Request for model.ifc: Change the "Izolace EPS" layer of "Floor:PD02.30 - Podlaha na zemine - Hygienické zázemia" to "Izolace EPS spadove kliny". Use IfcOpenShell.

First a look at what the model holds.

```python
import ifcopenshell
import ifcopenshell.util.element

model = ifcopenshell.open("model.ifc")
print(model.schema)
for layer_set in model.by_type("IfcMaterialLayerSet"):
    if layer_set.LayerSetName == "Floor:PD02.30 - Podlaha na zemine - Hygienické zázemia":
        for layer in layer_set.MaterialLayers:
            print(layer.id(), layer.Material and layer.Material.Name, layer.LayerThickness, sep=" | ")
        print(len(ifcopenshell.util.element.get_elements_by_material(model, layer_set)), "elements and types use it")
print(sorted(m.Name for m in model.by_type("IfcMaterial") if m.Name)[:60])
```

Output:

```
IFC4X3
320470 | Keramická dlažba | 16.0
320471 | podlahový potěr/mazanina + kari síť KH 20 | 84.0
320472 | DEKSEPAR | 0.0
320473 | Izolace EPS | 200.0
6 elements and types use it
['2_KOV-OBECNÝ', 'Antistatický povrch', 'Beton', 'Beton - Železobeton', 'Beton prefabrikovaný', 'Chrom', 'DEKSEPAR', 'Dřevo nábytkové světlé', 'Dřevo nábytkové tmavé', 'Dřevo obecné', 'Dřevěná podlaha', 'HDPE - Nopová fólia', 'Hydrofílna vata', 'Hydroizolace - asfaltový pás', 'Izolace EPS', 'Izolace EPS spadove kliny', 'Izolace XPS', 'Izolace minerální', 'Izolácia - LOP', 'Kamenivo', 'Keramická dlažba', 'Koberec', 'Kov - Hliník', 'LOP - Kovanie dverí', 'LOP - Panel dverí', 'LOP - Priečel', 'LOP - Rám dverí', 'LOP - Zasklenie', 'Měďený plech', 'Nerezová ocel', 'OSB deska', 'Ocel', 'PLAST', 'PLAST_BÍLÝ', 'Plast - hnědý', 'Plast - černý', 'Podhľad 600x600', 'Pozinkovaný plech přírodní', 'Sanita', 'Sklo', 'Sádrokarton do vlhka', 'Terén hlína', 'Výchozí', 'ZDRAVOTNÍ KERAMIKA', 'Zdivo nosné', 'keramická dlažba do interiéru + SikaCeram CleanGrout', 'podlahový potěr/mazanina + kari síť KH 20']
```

```python
import ifcopenshell
import ifcopenshell.api.material

model = ifcopenshell.open("model.ifc")

layer_set = next(s for s in model.by_type("IfcMaterialLayerSet") if s.LayerSetName == "Floor:PD02.30 - Podlaha na zemine - Hygienické zázemia")
layer = next(l for l in layer_set.MaterialLayers if l.Material and l.Material.Name == "Izolace EPS")
material = next(m for m in model.by_type("IfcMaterial") if m.Name == "Izolace EPS spadove kliny")

# Point this one layer at the other material; renaming the old one would change it everywhere.
ifcopenshell.api.material.edit_layer(model, layer=layer, attributes={"Name": material.Name}, material=material)

print([l.Material.Name if l.Material else None for l in layer_set.MaterialLayers])

model.write("model-out.ifc")
```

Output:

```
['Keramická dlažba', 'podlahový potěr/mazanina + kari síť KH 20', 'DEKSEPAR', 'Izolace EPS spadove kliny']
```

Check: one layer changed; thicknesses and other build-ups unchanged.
